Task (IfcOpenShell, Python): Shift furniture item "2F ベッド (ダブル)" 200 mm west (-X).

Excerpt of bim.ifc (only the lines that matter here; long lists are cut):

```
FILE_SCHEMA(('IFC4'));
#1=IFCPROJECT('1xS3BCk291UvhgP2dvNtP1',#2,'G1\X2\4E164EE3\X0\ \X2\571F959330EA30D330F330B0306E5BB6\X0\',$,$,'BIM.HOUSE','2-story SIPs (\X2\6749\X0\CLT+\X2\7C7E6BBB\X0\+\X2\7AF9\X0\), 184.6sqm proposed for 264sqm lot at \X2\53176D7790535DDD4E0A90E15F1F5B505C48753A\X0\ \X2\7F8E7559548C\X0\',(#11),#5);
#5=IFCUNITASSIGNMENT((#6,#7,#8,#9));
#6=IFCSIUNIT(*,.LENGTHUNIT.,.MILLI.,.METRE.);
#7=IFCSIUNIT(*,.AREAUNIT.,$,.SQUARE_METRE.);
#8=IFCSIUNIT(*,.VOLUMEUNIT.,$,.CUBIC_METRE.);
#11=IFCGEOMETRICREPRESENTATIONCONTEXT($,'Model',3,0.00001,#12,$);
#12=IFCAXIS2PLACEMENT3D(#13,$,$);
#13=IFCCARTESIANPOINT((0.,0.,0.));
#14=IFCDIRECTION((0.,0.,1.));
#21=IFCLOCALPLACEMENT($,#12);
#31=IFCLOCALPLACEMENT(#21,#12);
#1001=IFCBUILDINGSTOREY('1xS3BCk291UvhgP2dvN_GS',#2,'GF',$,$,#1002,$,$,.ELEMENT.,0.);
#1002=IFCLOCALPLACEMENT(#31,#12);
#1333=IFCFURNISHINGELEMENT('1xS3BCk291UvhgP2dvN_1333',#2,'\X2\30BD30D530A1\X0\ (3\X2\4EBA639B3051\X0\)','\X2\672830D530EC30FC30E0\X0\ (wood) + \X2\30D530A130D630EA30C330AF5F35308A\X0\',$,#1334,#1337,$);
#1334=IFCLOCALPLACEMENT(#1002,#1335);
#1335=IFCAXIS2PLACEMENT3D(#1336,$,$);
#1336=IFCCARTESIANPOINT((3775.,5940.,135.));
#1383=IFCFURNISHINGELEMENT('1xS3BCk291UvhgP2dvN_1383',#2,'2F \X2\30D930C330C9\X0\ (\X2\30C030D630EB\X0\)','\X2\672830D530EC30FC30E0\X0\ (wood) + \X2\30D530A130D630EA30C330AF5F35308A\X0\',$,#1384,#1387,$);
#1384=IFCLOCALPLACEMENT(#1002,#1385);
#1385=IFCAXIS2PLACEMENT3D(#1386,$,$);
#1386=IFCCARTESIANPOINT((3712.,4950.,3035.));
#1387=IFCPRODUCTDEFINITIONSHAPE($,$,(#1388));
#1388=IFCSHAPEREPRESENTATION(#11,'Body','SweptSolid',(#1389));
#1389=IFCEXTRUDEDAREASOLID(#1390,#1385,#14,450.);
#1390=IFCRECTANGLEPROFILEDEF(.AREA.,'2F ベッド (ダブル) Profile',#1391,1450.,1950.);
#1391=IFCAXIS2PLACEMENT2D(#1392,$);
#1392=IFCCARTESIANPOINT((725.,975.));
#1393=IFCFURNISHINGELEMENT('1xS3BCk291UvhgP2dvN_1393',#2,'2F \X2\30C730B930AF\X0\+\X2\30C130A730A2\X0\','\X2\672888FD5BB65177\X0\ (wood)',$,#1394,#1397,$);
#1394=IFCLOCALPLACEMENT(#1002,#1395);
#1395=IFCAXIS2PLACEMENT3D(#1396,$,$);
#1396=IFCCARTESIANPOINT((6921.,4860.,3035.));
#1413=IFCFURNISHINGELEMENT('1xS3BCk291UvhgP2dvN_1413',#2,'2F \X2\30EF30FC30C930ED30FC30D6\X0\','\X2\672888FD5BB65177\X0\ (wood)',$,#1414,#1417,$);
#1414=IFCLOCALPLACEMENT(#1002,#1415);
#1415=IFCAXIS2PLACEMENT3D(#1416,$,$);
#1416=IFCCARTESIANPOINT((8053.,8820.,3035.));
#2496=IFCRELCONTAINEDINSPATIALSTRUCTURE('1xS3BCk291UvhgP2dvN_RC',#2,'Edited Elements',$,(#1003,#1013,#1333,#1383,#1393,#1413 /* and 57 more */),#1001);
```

```python
import ifcopenshell
import ifcopenshell.api.geometry
import ifcopenshell.util.placement
import ifcopenshell.util.unit

model = ifcopenshell.open("bim.ifc")
unit_scale = ifcopenshell.util.unit.calculate_unit_scale(model)

item = model.by_guid("1xS3BCk291UvhgP2dvN_1383")
matrix = ifcopenshell.util.placement.get_local_placement(item.ObjectPlacement)
matrix[0, 3] -= 0.2 / unit_scale
ifcopenshell.api.geometry.edit_object_placement(model, product=item, matrix=matrix, is_si=False)

print(ifcopenshell.util.placement.get_local_placement(item.ObjectPlacement).round(3) + 0.0)

model.write("bim_edited.ifc")
```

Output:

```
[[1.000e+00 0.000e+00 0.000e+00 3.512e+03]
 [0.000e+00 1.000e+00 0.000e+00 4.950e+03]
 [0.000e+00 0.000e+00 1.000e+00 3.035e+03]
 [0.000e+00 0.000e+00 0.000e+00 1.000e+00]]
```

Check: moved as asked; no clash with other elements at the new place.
